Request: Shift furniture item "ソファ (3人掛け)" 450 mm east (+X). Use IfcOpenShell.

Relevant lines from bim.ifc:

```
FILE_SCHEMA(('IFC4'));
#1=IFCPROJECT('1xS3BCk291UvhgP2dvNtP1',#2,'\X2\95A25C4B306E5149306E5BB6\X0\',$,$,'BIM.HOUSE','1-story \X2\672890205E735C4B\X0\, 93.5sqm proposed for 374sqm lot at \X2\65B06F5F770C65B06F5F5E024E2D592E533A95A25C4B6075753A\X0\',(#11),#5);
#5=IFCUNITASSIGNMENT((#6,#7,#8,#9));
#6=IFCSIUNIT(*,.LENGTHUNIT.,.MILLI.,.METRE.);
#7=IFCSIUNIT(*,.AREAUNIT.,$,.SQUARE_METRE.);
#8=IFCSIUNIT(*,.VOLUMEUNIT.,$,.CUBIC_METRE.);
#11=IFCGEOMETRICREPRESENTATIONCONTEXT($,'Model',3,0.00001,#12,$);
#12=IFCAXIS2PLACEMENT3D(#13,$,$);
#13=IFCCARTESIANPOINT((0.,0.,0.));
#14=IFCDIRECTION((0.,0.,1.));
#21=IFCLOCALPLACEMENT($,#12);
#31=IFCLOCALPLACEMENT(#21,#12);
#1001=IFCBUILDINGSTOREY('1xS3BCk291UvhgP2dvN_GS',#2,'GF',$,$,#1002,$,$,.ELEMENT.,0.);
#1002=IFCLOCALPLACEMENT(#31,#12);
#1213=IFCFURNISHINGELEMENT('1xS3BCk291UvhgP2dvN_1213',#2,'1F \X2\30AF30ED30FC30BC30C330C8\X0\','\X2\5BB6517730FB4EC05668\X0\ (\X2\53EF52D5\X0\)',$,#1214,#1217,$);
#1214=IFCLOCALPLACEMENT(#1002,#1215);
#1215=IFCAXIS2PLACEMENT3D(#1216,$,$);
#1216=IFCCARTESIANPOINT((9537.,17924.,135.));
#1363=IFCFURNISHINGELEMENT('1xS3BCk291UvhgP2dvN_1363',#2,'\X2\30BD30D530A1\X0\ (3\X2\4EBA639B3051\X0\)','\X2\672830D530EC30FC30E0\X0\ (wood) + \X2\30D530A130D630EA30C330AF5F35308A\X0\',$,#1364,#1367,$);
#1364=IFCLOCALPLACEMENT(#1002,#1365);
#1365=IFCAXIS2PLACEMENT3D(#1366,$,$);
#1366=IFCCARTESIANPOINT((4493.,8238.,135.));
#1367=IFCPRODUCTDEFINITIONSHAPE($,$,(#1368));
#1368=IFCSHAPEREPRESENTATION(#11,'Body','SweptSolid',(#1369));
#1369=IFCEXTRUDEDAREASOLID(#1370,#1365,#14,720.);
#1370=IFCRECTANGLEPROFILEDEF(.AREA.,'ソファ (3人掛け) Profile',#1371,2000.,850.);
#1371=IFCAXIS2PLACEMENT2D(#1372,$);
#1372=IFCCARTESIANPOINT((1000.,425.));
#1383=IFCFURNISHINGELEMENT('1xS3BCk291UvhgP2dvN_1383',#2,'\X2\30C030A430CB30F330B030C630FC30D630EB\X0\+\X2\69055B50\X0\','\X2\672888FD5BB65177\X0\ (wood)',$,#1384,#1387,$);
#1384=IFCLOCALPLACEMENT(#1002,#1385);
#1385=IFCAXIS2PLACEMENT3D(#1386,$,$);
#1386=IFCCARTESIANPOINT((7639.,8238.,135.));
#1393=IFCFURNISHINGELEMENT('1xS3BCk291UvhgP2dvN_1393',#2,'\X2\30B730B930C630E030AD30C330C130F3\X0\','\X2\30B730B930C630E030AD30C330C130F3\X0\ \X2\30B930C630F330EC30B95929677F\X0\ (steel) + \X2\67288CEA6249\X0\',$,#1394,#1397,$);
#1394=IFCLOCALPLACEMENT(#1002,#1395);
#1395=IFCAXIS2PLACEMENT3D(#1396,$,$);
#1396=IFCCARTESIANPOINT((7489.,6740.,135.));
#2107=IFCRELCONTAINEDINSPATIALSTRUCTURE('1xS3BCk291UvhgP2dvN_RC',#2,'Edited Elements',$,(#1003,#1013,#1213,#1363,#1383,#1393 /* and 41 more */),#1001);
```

```python
import ifcopenshell
import ifcopenshell.api.geometry
import ifcopenshell.util.placement

model = ifcopenshell.open("bim.ifc")

item = model.by_guid("1xS3BCk291UvhgP2dvN_1363")
matrix = ifcopenshell.util.placement.get_local_placement(item.ObjectPlacement)
matrix[0, 3] += 450.0
ifcopenshell.api.geometry.edit_object_placement(model, product=item, matrix=matrix, is_si=False)

print(ifcopenshell.util.placement.get_local_placement(item.ObjectPlacement).round(3) + 0.0)

model.write("bim_rev.ifc")
```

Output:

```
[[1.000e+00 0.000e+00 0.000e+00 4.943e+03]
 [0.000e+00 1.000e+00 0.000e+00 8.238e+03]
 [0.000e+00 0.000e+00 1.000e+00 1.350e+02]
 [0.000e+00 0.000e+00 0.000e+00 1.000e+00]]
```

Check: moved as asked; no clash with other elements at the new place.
